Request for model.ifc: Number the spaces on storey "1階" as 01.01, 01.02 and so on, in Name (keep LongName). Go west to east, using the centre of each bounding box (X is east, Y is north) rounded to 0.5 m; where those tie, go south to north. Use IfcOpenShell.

First a look at what the model holds.

```python
import ifcopenshell
import ifcopenshell.util.element
import ifcopenshell.util.placement

model = ifcopenshell.open("model.ifc")
print(model.schema)
storey = next(s for s in model.by_type("IfcBuildingStorey") if s.Name == "1階")
spaces = [e for e in ifcopenshell.util.element.get_decomposition(storey) if e.is_a("IfcSpace")]
for e in sorted(spaces, key=lambda e: e.id()):
    origin = ifcopenshell.util.placement.get_local_placement(e.ObjectPlacement)[:3, 3]
    print(e.id(), e.Name, e.LongName, origin.round(2) + 0.0, sep=" | ")
```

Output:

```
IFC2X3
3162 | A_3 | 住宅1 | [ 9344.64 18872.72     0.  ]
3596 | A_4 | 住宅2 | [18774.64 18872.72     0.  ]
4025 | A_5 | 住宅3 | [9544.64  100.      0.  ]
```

```python
import ifcopenshell
import ifcopenshell.geom
import ifcopenshell.util.element
import ifcopenshell.util.shape

model = ifcopenshell.open("model.ifc")
settings = ifcopenshell.geom.settings()
settings.set("use-world-coords", True)


def centre(element):
    shape = ifcopenshell.geom.create_shape(settings, element)
    return ifcopenshell.util.shape.get_bbox_centroid(shape.geometry)


storey = next(s for s in model.by_type("IfcBuildingStorey") if s.Name == "1階")
spaces = [e for e in ifcopenshell.util.element.get_decomposition(storey) if e.is_a("IfcSpace")]

# Insertion points can sit at a corner or the storey origin, so sort by the geometry (in metres).
centres = {e: centre(e) for e in spaces}
spaces.sort(key=lambda e: (round(centres[e][0] / 0.5), centres[e][1]))

for i, e in enumerate(spaces, start=1):
    number = f"01.{i:02d}"
    e.Name = number
    print(e.id(), number)

model.write("model_edited.ifc")
```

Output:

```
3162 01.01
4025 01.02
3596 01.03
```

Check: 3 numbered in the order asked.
